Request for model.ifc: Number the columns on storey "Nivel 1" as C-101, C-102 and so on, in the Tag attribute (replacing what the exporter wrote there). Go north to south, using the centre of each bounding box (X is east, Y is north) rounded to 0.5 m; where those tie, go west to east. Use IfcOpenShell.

First a look at what the model holds.

```python
import ifcopenshell
import ifcopenshell.util.element
import ifcopenshell.util.placement

model = ifcopenshell.open("model.ifc")
print(model.schema)
storey = next(s for s in model.by_type("IfcBuildingStorey") if s.Name == "Nivel 1")
columns = [e for e in ifcopenshell.util.element.get_decomposition(storey) if e.is_a("IfcColumn")]
for e in sorted(columns, key=lambda e: e.id()):
    origin = ifcopenshell.util.placement.get_local_placement(e.ObjectPlacement)[:3, 3]
    print(e.id(), e.Tag, e.Name, origin.round(2) + 0.0, sep=" | ")
```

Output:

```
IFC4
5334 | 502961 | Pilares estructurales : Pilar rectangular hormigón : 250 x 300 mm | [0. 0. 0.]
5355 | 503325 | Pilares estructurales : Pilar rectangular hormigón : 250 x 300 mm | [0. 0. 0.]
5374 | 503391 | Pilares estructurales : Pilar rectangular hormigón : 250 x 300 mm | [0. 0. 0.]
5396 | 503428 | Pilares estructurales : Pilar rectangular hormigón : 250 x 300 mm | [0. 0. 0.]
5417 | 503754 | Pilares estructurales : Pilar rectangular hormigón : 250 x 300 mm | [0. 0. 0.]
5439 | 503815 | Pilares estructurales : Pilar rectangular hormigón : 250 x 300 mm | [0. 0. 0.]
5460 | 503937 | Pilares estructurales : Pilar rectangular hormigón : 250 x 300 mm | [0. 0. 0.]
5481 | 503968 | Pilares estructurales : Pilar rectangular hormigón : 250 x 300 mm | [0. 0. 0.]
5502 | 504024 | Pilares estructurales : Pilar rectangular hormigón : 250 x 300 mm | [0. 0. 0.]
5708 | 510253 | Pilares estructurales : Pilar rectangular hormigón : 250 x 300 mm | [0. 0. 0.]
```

```python
import ifcopenshell
import ifcopenshell.geom
import ifcopenshell.util.element
import ifcopenshell.util.shape

model = ifcopenshell.open("model.ifc")
settings = ifcopenshell.geom.settings()
settings.set("use-world-coords", True)


def centre(element):
    shape = ifcopenshell.geom.create_shape(settings, element)
    return ifcopenshell.util.shape.get_bbox_centroid(shape.geometry)


storey = next(s for s in model.by_type("IfcBuildingStorey") if s.Name == "Nivel 1")
columns = [e for e in ifcopenshell.util.element.get_decomposition(storey) if e.is_a("IfcColumn")]

# Insertion points can sit at a corner or the storey origin, so sort by the geometry (in metres).
centres = {e: centre(e) for e in columns}
columns.sort(key=lambda e: (-round(centres[e][1] / 0.5), centres[e][0]))

for i, e in enumerate(columns, start=1):
    number = f"C-1{i:02d}"
    e.Tag = number
    print(e.id(), number)

model.write("model_updated.ifc")
```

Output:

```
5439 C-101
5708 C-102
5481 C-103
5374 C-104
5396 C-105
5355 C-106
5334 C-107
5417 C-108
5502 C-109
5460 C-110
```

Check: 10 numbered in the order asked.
